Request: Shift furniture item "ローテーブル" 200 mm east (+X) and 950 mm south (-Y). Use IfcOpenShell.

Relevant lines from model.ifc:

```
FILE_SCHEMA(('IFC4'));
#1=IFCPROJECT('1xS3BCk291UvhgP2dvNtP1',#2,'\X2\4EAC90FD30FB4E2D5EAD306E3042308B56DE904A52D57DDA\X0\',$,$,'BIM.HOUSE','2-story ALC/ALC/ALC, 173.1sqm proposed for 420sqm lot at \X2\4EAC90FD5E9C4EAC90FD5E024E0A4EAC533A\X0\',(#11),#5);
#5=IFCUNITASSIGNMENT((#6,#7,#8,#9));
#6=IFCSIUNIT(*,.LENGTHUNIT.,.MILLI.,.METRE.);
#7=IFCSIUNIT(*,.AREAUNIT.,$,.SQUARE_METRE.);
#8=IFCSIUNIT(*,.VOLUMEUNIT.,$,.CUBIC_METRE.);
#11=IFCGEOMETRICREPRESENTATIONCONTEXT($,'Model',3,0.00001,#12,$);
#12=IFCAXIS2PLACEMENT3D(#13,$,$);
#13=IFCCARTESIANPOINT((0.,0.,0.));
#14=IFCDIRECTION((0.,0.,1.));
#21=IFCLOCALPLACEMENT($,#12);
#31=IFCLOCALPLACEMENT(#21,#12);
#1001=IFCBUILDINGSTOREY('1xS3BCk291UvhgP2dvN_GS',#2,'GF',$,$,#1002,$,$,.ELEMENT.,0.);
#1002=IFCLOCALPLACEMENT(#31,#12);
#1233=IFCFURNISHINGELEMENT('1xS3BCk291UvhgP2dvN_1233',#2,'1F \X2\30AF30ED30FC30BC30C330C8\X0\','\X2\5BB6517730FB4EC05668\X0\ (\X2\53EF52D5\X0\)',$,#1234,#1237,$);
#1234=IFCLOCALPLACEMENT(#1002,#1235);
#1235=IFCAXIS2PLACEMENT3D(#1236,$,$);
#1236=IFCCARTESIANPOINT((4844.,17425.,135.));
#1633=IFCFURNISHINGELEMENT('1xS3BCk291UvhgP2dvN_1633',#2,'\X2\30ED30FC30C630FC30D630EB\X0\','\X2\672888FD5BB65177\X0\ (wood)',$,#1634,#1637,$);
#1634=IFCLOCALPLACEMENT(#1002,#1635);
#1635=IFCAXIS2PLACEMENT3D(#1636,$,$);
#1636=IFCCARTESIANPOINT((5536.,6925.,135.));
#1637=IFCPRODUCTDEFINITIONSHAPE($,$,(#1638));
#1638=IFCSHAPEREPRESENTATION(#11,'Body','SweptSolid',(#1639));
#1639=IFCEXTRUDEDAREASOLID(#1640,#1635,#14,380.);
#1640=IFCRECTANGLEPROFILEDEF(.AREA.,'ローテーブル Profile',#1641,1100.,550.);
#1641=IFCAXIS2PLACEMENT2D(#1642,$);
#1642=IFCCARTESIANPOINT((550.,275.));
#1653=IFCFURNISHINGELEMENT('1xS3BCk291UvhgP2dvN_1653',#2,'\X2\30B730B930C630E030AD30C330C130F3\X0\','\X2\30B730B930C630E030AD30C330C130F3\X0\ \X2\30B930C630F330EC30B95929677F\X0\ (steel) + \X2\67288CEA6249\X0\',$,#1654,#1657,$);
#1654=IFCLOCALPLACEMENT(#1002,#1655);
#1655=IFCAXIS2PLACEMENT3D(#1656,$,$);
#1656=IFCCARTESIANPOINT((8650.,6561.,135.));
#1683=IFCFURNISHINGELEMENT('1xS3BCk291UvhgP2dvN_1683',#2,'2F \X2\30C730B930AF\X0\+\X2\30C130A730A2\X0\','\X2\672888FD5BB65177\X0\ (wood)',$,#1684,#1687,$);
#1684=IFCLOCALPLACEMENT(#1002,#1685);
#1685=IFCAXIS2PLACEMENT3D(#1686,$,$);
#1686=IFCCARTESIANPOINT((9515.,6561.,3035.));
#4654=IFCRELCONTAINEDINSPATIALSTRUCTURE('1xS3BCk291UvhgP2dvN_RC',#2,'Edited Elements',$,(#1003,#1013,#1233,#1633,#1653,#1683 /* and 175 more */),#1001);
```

```python
import ifcopenshell
import ifcopenshell.api.geometry
import ifcopenshell.util.placement
import ifcopenshell.util.unit

model = ifcopenshell.open("model.ifc")
unit_scale = ifcopenshell.util.unit.calculate_unit_scale(model)

item = model.by_guid("1xS3BCk291UvhgP2dvN_1633")
matrix = ifcopenshell.util.placement.get_local_placement(item.ObjectPlacement)
matrix[0, 3] += 0.2 / unit_scale
matrix[1, 3] -= 0.95 / unit_scale
ifcopenshell.api.geometry.edit_object_placement(model, product=item, matrix=matrix, is_si=False)

print(ifcopenshell.util.placement.get_local_placement(item.ObjectPlacement).round(3) + 0.0)

model.write("model_v2.ifc")
```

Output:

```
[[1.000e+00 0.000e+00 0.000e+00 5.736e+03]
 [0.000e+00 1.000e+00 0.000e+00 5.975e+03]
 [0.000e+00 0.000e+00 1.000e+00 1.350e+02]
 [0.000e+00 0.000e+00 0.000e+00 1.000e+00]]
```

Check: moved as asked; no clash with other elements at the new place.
